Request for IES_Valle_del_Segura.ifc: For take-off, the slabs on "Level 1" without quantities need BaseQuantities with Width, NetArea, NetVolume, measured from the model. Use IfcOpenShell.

First a look at what the model holds.

```python
import ifcopenshell
import ifcopenshell.util.element
import ifcopenshell.util.unit

model = ifcopenshell.open("IES_Valle_del_Segura.ifc")
print(model.schema)
for unit_type in ("LENGTHUNIT", "AREAUNIT", "VOLUMEUNIT"):
    print(unit_type, ifcopenshell.util.unit.calculate_unit_scale(model, unit_type))
storey = next(s for s in model.by_type("IfcBuildingStorey") if s.Name == "Level 1")
slabs = [e for e in ifcopenshell.util.element.get_decomposition(storey) if e.is_a("IfcSlab")]
for e in sorted(slabs, key=lambda e: e.id()):
    print(e.id(), e.is_a(), e.Name, list(ifcopenshell.util.element.get_psets(e, qtos_only=True)), sep=" | ")
```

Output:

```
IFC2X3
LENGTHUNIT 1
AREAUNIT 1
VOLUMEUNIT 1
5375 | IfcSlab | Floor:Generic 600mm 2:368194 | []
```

```python
import ifcopenshell
import ifcopenshell.api.pset
import ifcopenshell.geom
import ifcopenshell.util.element
import ifcopenshell.util.shape
import ifcopenshell.util.unit

model = ifcopenshell.open("IES_Valle_del_Segura.ifc")
unit_scale = ifcopenshell.util.unit.calculate_unit_scale(model)
area_scale = ifcopenshell.util.unit.calculate_unit_scale(model, "AREAUNIT")
volume_scale = ifcopenshell.util.unit.calculate_unit_scale(model, "VOLUMEUNIT")
settings = ifcopenshell.geom.settings()

storey = next(s for s in model.by_type("IfcBuildingStorey") if s.Name == "Level 1")
slabs = [e for e in ifcopenshell.util.element.get_decomposition(storey) if e.is_a("IfcSlab")]

for e in sorted(slabs, key=lambda e: e.id()):
    if ifcopenshell.util.element.get_psets(e, qtos_only=True, should_inherit=False):
        continue
    # Geometry comes back in metres, in the element's own axes.
    shape = ifcopenshell.geom.create_shape(settings, e)
    values = {
        "Width": ifcopenshell.util.shape.get_z(shape.geometry) / unit_scale,
        "NetArea": ifcopenshell.util.shape.get_footprint_area(shape.geometry) / area_scale,
        "NetVolume": ifcopenshell.util.shape.get_volume(shape.geometry) / volume_scale,
    }
    qto = ifcopenshell.api.pset.add_qto(model, product=e, name="BaseQuantities")
    ifcopenshell.api.pset.edit_qto(model, qto=qto, properties=values)
    print(e.id(), {k: round(v, 3) for k, v in values.items()})

model.write("IES_Valle_del_Segura_v2.ifc")
```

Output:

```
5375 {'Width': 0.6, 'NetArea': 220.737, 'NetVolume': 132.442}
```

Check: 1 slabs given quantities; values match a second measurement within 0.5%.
